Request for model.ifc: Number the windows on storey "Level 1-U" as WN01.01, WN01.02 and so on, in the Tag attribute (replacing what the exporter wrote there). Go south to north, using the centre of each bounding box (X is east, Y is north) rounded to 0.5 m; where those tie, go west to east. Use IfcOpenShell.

First a look at what the model holds.

```python
import ifcopenshell
import ifcopenshell.util.element
import ifcopenshell.util.placement

model = ifcopenshell.open("model.ifc")
print(model.schema)
storey = next(s for s in model.by_type("IfcBuildingStorey") if s.Name == "Level 1-U")
windows = [e for e in ifcopenshell.util.element.get_decomposition(storey) if e.is_a("IfcWindow")]
for e in sorted(windows, key=lambda e: e.id()):
    origin = ifcopenshell.util.placement.get_local_placement(e.ObjectPlacement)[:3, 3]
    print(e.id(), e.Tag, e.Name, origin.round(2) + 0.0, sep=" | ")
```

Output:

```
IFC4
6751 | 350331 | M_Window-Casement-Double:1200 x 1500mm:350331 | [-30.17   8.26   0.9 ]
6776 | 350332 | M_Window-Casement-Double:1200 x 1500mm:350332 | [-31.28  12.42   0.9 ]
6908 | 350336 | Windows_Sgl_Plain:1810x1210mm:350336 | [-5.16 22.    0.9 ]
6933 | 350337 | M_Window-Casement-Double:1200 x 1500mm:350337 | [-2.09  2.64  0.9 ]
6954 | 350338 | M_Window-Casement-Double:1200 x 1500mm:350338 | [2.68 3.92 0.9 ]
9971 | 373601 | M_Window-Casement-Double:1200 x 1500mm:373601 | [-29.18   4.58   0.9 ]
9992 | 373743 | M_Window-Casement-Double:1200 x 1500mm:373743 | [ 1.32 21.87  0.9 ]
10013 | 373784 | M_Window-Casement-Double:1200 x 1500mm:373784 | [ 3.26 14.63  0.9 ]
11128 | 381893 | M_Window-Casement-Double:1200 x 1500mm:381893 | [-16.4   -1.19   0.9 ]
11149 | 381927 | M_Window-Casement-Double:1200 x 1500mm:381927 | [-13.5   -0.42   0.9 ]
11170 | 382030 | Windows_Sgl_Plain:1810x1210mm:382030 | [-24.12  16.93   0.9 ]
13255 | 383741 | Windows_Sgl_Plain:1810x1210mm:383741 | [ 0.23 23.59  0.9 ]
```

```python
import ifcopenshell
import ifcopenshell.geom
import ifcopenshell.util.element
import ifcopenshell.util.shape

model = ifcopenshell.open("model.ifc")
settings = ifcopenshell.geom.settings()
settings.set("use-world-coords", True)


def centre(element):
    shape = ifcopenshell.geom.create_shape(settings, element)
    return ifcopenshell.util.shape.get_bbox_centroid(shape.geometry)


storey = next(s for s in model.by_type("IfcBuildingStorey") if s.Name == "Level 1-U")
windows = [e for e in ifcopenshell.util.element.get_decomposition(storey) if e.is_a("IfcWindow")]

# Insertion points can sit at a corner or the storey origin, so sort by the geometry (in metres).
centres = {e: centre(e) for e in windows}
windows.sort(key=lambda e: (round(centres[e][1] / 0.5), centres[e][0]))

for i, e in enumerate(windows, start=1):
    number = f"WN01.{i:02d}"
    e.Tag = number
    print(e.id(), number)

model.write("model_edited.ifc")
```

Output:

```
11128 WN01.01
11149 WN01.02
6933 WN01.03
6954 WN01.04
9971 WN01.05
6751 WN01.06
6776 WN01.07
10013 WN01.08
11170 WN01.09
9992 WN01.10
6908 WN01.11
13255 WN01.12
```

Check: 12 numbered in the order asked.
